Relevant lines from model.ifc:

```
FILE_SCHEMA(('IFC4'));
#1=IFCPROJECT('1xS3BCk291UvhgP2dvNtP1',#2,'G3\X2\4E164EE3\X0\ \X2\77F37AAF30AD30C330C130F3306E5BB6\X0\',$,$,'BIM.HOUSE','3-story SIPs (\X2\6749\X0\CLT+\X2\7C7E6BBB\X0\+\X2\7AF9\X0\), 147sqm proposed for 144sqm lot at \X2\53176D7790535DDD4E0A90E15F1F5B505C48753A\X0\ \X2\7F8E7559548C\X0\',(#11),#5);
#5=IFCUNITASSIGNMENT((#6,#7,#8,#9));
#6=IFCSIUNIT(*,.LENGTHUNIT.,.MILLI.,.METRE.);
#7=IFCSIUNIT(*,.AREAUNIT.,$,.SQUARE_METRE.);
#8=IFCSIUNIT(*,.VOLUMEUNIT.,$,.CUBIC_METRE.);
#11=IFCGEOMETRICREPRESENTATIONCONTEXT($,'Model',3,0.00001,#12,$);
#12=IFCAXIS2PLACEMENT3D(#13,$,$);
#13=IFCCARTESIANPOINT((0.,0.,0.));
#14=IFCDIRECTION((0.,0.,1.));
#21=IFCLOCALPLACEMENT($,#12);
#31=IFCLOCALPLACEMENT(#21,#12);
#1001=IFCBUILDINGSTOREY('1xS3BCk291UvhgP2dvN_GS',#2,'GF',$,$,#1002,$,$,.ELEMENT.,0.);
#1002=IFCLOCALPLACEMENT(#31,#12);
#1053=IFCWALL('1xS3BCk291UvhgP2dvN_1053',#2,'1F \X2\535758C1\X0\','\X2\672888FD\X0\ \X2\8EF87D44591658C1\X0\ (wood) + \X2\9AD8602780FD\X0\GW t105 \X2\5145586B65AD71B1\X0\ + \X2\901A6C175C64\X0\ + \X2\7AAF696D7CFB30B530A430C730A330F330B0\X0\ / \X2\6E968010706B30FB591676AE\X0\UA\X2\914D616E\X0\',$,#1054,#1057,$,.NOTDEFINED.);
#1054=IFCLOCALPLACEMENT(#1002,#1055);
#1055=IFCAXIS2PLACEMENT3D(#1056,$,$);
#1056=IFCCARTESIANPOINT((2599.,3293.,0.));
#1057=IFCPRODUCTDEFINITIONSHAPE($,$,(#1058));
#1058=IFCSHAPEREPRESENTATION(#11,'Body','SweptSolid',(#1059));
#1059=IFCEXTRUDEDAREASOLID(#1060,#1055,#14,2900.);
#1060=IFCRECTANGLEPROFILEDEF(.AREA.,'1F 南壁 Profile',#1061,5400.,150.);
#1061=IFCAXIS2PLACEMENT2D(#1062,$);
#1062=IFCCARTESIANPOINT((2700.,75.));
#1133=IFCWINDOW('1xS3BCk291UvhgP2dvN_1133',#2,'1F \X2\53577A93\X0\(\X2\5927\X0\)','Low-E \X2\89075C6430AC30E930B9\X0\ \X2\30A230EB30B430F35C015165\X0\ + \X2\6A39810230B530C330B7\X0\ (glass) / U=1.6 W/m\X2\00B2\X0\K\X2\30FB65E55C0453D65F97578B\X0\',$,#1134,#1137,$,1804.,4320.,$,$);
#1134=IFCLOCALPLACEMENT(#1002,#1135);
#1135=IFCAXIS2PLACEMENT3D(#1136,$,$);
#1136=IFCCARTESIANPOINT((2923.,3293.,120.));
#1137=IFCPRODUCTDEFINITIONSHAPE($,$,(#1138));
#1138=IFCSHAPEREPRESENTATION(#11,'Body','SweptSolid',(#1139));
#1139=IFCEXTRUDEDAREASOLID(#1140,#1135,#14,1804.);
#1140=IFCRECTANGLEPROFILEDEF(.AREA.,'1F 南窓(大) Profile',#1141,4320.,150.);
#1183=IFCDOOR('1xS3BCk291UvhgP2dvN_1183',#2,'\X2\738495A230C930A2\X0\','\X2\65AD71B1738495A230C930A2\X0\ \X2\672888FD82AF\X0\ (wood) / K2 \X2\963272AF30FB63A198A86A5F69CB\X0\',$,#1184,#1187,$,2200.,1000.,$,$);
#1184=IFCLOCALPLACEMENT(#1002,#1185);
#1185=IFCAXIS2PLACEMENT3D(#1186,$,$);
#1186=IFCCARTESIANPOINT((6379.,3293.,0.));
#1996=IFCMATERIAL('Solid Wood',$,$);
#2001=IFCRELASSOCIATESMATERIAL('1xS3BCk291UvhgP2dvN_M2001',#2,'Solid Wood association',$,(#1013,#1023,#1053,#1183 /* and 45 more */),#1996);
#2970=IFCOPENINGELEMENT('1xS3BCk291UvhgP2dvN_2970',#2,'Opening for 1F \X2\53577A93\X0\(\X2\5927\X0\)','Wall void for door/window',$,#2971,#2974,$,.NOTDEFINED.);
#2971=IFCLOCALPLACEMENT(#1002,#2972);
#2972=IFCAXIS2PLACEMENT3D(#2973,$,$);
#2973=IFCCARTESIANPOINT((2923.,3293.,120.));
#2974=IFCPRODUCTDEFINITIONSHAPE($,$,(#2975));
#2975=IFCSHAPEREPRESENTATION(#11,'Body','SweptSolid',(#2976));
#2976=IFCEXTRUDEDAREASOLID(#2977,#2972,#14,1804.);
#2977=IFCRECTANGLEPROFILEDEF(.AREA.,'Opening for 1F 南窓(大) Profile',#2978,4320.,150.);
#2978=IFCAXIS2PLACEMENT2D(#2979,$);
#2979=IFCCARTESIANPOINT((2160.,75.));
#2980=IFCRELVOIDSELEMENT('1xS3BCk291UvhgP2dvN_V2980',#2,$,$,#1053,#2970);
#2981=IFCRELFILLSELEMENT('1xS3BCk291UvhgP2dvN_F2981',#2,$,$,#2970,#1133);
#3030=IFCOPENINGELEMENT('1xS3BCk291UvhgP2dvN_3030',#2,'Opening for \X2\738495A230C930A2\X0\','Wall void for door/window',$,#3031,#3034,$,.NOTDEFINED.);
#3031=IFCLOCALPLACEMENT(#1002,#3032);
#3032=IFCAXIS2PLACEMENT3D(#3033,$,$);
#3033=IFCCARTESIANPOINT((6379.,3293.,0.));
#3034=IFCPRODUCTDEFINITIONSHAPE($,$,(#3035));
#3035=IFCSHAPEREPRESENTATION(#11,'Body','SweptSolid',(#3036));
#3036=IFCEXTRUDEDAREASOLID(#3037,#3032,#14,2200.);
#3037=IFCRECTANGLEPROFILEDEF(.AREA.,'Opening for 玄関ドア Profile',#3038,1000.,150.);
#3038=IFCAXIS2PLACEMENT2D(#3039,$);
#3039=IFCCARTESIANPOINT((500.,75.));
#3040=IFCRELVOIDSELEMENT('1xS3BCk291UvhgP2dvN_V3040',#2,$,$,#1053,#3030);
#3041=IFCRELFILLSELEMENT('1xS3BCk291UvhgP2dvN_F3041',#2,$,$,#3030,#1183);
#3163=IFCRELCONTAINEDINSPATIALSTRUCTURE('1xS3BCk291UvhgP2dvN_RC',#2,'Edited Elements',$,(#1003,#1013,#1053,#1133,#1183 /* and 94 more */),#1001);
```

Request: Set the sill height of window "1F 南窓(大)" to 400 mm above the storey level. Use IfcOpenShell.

```python
import numpy as np
import ifcopenshell
import ifcopenshell.api.geometry
import ifcopenshell.geom
import ifcopenshell.util.element
import ifcopenshell.util.placement
import ifcopenshell.util.shape
import ifcopenshell.util.unit

model = ifcopenshell.open("model.ifc")
unit_scale = ifcopenshell.util.unit.calculate_unit_scale(model)

window = model.by_guid("1xS3BCk291UvhgP2dvN_1133")
opening = window.FillsVoids[0].RelatingOpeningElement
storey = ifcopenshell.util.element.get_container(window, ifc_class="IfcBuildingStorey")
level = ifcopenshell.util.placement.get_local_placement(storey.ObjectPlacement)[2, 3]

# The opening's origin need not be at the sill, so measure its lowest point.
shape = ifcopenshell.geom.create_shape(ifcopenshell.geom.settings(), opening)
bottom = ifcopenshell.util.shape.get_shape_bottom_elevation(shape, shape.geometry) / unit_scale
dz = level + 0.4 / unit_scale - bottom

shift = np.array([0.0, 0.0, dz])
# The window is not placed relative to its opening, so move both.
for product in (opening, window):
    matrix = ifcopenshell.util.placement.get_local_placement(product.ObjectPlacement)
    matrix[:3, 3] += shift
    ifcopenshell.api.geometry.edit_object_placement(model, product=product, matrix=matrix, is_si=False)

print(f"moved by {dz * unit_scale:+.3f} m")

model.write("model_edited.ifc")
```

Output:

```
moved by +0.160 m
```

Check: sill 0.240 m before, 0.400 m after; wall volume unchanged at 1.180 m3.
